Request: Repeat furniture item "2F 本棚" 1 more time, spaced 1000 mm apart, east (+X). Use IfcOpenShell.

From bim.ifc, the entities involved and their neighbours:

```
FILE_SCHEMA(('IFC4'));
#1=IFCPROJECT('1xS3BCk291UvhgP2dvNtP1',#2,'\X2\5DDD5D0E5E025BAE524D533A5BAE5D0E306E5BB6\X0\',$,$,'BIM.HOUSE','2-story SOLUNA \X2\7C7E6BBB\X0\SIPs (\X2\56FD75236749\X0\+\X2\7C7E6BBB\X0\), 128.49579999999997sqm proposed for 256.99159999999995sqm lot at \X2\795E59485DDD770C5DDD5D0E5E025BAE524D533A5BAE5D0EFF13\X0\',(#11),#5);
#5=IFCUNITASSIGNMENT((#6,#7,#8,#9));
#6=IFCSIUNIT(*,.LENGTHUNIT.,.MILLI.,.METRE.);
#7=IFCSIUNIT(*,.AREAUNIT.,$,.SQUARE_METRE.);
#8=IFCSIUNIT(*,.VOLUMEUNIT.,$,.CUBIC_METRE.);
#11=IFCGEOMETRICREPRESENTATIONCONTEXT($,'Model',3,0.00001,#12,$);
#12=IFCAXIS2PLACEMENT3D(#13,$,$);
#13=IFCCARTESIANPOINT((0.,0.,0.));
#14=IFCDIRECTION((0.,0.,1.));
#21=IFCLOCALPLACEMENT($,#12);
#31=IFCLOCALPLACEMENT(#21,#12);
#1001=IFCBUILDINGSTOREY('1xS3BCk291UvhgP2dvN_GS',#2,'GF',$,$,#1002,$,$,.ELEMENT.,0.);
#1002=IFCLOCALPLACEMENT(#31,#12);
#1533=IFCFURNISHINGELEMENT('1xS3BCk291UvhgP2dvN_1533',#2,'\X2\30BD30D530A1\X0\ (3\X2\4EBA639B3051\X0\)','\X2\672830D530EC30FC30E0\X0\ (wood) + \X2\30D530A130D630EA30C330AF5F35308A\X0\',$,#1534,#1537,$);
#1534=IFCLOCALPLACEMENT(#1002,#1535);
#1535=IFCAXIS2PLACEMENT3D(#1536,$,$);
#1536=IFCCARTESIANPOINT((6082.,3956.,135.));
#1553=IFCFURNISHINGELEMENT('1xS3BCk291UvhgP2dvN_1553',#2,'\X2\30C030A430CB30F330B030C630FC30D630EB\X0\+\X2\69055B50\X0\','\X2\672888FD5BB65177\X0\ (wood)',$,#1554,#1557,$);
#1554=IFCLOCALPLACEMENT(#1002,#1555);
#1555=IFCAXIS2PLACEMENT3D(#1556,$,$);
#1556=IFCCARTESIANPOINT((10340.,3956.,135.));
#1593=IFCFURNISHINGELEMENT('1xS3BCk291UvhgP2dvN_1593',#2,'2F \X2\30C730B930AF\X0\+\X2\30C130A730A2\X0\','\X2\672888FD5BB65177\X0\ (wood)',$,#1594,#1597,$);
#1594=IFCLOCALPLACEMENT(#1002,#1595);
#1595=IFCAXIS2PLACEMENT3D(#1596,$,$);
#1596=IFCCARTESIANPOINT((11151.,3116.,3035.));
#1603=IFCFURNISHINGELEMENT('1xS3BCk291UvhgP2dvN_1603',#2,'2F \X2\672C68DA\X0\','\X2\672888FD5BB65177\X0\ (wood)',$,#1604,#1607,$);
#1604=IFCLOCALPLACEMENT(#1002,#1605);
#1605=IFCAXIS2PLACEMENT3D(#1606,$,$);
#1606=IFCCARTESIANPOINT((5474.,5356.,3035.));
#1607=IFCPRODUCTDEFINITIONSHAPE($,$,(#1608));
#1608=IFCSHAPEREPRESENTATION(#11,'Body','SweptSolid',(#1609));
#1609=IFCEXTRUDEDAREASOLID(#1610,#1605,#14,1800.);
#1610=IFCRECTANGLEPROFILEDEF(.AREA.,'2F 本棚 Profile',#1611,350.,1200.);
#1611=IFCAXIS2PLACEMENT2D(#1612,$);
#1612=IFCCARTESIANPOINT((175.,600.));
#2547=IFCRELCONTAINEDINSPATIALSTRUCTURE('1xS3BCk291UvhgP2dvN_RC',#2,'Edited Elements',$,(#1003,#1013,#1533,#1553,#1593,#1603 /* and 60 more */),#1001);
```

```python
import numpy as np
import ifcopenshell
import ifcopenshell.api.geometry
import ifcopenshell.api.root
import ifcopenshell.util.element
import ifcopenshell.util.placement
import ifcopenshell.util.unit

model = ifcopenshell.open("bim.ifc")
unit_scale = ifcopenshell.util.unit.calculate_unit_scale(model)


def reuse_history(source, copy):
    """copy_class also copies each property set's owner history, people and application; keep the originals."""
    for rel in copy.IsDefinedBy:
        if rel.is_a("IfcRelDefinesByProperties") and (history := rel.RelatingPropertyDefinition.OwnerHistory):
            rel.RelatingPropertyDefinition.OwnerHistory = source.OwnerHistory
            ifcopenshell.util.element.remove_deep2(model, history)


source = model.by_guid("1xS3BCk291UvhgP2dvN_1603")
base = ifcopenshell.util.placement.get_local_placement(source.ObjectPlacement)
step = np.array([1.0, 0.0, 0.0]) * 1 / unit_scale

for i in range(1, 2):
    copy = ifcopenshell.api.root.copy_class(model, product=source)
    copy.Representation = ifcopenshell.util.element.copy_deep(
        model, source.Representation, exclude=["IfcGeometricRepresentationContext", "IfcRepresentationMap"]
    )
    reuse_history(source, copy)
    matrix = base.copy()
    matrix[:3, 3] += i * step
    print("added at", matrix[:3, 3].round(3) + 0.0)
    ifcopenshell.api.geometry.edit_object_placement(model, product=copy, matrix=matrix, is_si=False)

model.write("bim-out.ifc")
```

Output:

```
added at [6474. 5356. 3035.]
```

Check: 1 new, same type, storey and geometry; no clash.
